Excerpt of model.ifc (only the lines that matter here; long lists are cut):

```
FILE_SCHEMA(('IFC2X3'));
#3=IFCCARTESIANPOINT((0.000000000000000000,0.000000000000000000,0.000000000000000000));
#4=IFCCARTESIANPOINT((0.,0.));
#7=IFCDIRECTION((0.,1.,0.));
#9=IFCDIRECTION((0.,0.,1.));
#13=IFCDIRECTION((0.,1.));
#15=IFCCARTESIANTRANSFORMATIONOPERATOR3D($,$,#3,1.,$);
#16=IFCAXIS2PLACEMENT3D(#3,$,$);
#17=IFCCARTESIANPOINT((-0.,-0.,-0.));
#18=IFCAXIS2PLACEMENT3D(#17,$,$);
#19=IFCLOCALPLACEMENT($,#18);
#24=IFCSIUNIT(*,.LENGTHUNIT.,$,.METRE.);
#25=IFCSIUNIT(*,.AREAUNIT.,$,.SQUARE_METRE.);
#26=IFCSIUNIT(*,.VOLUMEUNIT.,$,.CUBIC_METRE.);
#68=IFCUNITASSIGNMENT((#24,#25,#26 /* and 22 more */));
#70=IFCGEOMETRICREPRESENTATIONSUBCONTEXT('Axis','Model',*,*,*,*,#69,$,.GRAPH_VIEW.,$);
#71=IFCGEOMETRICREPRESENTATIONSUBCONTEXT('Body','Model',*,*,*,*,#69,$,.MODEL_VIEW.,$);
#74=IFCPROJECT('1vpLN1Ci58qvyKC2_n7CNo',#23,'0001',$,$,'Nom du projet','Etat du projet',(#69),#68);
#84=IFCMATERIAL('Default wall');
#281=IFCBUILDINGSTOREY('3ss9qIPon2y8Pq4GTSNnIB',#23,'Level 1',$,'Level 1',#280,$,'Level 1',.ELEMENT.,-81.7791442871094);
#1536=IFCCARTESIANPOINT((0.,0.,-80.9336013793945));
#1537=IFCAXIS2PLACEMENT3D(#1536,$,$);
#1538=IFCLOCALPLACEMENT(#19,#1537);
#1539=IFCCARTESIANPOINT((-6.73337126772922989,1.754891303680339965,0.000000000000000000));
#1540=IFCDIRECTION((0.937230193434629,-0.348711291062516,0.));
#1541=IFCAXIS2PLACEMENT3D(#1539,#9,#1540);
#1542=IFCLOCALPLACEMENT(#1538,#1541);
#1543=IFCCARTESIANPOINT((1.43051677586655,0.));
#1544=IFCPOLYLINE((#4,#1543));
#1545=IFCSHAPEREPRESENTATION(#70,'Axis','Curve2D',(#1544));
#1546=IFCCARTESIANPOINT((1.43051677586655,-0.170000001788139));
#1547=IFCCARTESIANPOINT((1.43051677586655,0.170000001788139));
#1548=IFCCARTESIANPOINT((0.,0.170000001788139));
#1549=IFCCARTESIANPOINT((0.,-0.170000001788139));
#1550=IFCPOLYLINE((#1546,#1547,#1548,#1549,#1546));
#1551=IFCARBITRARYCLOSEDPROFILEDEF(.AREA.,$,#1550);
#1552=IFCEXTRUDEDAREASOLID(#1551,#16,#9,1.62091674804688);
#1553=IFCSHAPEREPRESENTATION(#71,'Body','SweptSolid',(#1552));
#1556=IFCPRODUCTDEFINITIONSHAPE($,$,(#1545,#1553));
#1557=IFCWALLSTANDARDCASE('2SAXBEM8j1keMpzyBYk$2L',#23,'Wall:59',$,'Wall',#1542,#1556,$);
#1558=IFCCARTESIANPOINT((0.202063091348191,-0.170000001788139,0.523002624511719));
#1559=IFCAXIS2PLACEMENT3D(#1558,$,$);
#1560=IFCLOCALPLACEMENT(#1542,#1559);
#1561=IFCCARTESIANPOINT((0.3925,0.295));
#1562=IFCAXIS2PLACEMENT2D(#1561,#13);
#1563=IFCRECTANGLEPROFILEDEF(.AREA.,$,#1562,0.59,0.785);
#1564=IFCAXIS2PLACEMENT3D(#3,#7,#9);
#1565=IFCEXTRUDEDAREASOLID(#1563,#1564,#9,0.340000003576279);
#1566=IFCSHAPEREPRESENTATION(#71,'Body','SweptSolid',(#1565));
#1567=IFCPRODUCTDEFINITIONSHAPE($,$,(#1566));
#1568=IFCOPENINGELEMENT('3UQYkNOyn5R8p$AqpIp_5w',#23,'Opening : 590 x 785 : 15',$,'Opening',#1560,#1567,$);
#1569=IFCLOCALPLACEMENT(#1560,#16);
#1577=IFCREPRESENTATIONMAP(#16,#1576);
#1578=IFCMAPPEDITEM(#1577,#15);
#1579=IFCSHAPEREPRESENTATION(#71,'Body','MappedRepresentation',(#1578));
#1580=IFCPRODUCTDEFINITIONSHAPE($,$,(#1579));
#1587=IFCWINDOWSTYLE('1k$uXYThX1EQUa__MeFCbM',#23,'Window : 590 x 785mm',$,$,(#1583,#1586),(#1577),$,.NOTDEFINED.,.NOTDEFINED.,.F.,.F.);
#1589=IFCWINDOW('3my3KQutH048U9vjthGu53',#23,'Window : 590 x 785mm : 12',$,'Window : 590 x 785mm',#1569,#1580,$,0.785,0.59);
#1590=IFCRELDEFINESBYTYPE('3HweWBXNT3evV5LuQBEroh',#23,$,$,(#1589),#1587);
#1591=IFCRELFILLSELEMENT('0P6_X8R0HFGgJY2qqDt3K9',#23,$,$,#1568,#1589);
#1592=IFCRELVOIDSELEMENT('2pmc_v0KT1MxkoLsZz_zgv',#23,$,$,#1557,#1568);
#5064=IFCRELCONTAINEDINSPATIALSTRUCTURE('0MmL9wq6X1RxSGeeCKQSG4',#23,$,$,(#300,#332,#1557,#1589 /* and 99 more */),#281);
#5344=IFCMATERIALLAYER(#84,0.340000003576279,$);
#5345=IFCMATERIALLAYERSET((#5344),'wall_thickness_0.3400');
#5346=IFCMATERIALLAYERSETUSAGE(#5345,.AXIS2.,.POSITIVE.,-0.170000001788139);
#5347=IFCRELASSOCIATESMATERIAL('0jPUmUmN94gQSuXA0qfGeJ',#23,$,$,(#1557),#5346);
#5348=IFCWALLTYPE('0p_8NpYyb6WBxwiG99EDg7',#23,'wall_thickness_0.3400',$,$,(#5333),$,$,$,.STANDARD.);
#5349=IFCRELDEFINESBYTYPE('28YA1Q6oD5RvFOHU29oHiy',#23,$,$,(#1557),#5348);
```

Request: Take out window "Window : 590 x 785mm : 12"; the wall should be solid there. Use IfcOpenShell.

```python
import ifcopenshell
import ifcopenshell.api.feature
import ifcopenshell.api.root
import ifcopenshell.geom
import ifcopenshell.util.shape

model = ifcopenshell.open("model.ifc")
settings = ifcopenshell.geom.settings()


def volume(element):
    """Net volume in cubic metres, openings subtracted."""
    shape = ifcopenshell.geom.create_shape(settings, element)
    return ifcopenshell.util.shape.get_volume(shape.geometry)


window = model.by_guid("3my3KQutH048U9vjthGu53")
opening = window.FillsVoids[0].RelatingOpeningElement
wall = opening.VoidsElements[0].RelatingBuildingElement
before = volume(wall)

ifcopenshell.api.root.remove_product(model, product=window)
ifcopenshell.api.feature.remove_feature(model, feature=opening)

after = volume(wall)

print(f"wall volume {before:.3f} -> {after:.3f} m3")

model.write("model_edited.ifc")
```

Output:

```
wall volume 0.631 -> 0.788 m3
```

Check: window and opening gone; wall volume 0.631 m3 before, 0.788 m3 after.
